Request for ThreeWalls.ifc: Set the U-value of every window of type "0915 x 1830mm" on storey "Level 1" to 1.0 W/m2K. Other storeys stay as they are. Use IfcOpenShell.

First a look at what the model holds.

```python
import ifcopenshell
import ifcopenshell.util.element

model = ifcopenshell.open("ThreeWalls.ifc")
print(model.schema)
storey = next(s for s in model.by_type("IfcBuildingStorey") if s.Name == "Level 1")
windows = [e for e in ifcopenshell.util.element.get_decomposition(storey) if e.is_a("IfcWindow")]
seen = {}
for e in windows:
    element_type = ifcopenshell.util.element.get_type(e)
    key = (element_type.Name if element_type != e and element_type else None, ifcopenshell.util.element.get_pset(e, "Pset_WindowCommon", "ThermalTransmittance"))
    seen[key] = seen.get(key, 0) + 1
for (name, value), count in sorted(seen.items(), key=str):
    print(count, "x", name, "|", value)
```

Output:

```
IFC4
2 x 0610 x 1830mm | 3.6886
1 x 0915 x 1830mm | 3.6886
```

```python
import ifcopenshell
import ifcopenshell.api.pset
import ifcopenshell.util.element

model = ifcopenshell.open("ThreeWalls.ifc")

storey = next(s for s in model.by_type("IfcBuildingStorey") if s.Name == "Level 1")
windows = [e for e in ifcopenshell.util.element.get_decomposition(storey) if e.is_a("IfcWindow")]

count = 0
for e in windows:
    element_type = ifcopenshell.util.element.get_type(e)
    if element_type in (None, e) or element_type.Name != "0915 x 1830mm":
        continue
    # add_pset returns the element's existing set when there is one.
    pset = ifcopenshell.api.pset.add_pset(model, product=e, name="Pset_WindowCommon")
    ifcopenshell.api.pset.edit_pset(model, pset=pset, properties={"ThermalTransmittance": 1.0})
    count += 1

print(count, "windows updated")

model.write("ThreeWalls-out.ifc")
```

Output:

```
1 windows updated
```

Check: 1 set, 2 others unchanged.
